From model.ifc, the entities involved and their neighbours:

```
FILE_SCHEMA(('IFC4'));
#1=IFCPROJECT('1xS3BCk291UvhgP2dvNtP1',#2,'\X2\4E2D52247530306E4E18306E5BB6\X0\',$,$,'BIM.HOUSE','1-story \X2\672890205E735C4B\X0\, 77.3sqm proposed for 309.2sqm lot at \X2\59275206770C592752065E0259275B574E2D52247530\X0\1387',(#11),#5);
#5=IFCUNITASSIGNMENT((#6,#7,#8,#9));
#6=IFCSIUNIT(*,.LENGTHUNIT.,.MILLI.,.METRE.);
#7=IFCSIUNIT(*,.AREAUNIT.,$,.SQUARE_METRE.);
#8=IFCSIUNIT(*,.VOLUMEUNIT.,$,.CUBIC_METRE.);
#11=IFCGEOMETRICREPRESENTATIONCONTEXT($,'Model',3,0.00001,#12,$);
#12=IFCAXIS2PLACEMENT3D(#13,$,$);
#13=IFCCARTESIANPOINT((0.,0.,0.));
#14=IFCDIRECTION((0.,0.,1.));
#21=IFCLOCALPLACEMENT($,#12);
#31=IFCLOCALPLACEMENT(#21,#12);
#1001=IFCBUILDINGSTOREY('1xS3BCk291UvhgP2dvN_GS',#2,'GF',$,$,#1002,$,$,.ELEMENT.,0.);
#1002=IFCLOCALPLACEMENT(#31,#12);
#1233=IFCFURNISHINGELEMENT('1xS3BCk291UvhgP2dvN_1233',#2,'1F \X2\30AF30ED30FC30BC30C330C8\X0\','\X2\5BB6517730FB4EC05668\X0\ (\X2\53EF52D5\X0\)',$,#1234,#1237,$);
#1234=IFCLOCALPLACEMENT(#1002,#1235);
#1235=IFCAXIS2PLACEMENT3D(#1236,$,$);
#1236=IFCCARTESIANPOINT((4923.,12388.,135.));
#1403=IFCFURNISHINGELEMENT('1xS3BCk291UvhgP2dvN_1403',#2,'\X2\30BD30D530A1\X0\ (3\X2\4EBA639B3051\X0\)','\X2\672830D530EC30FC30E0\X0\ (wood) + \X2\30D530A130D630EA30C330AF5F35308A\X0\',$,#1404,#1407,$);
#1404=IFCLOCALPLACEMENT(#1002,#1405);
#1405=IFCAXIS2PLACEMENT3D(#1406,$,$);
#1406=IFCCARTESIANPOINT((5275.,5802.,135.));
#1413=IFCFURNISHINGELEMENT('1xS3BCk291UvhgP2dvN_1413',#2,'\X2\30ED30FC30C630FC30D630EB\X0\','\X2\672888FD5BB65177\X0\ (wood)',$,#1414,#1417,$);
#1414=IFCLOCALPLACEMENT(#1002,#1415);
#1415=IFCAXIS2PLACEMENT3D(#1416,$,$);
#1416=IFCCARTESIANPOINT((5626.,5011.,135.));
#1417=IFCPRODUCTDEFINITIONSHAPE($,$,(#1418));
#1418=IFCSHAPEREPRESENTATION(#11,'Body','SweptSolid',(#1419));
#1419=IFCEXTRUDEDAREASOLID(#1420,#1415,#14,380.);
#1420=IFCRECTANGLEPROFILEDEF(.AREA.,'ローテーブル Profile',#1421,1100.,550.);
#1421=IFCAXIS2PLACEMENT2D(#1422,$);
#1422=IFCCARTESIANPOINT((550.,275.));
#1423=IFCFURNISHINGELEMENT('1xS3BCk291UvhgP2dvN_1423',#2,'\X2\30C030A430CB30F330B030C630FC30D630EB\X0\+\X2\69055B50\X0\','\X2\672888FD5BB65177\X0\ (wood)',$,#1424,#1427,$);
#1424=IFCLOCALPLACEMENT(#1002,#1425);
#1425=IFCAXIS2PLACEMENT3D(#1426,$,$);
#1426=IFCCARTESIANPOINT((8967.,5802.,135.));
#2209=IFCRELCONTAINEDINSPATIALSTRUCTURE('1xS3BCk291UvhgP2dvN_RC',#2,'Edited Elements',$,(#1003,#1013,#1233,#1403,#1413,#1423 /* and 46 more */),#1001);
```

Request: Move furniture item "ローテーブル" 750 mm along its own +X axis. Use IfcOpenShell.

```python
import ifcopenshell
import ifcopenshell.api.geometry
import ifcopenshell.util.placement

model = ifcopenshell.open("model.ifc")

item = model.by_id(1413)
matrix = ifcopenshell.util.placement.get_local_placement(item.ObjectPlacement)
matrix[:3, 3] += matrix[:3, 0] * 750.0
ifcopenshell.api.geometry.edit_object_placement(model, product=item, matrix=matrix, is_si=False)

print(ifcopenshell.util.placement.get_local_placement(item.ObjectPlacement).round(3) + 0.0)

model.write("model_edited.ifc")
```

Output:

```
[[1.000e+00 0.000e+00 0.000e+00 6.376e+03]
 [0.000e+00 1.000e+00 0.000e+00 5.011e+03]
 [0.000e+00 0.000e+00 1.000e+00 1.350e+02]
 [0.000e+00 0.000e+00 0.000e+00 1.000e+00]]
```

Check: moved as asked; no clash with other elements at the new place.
